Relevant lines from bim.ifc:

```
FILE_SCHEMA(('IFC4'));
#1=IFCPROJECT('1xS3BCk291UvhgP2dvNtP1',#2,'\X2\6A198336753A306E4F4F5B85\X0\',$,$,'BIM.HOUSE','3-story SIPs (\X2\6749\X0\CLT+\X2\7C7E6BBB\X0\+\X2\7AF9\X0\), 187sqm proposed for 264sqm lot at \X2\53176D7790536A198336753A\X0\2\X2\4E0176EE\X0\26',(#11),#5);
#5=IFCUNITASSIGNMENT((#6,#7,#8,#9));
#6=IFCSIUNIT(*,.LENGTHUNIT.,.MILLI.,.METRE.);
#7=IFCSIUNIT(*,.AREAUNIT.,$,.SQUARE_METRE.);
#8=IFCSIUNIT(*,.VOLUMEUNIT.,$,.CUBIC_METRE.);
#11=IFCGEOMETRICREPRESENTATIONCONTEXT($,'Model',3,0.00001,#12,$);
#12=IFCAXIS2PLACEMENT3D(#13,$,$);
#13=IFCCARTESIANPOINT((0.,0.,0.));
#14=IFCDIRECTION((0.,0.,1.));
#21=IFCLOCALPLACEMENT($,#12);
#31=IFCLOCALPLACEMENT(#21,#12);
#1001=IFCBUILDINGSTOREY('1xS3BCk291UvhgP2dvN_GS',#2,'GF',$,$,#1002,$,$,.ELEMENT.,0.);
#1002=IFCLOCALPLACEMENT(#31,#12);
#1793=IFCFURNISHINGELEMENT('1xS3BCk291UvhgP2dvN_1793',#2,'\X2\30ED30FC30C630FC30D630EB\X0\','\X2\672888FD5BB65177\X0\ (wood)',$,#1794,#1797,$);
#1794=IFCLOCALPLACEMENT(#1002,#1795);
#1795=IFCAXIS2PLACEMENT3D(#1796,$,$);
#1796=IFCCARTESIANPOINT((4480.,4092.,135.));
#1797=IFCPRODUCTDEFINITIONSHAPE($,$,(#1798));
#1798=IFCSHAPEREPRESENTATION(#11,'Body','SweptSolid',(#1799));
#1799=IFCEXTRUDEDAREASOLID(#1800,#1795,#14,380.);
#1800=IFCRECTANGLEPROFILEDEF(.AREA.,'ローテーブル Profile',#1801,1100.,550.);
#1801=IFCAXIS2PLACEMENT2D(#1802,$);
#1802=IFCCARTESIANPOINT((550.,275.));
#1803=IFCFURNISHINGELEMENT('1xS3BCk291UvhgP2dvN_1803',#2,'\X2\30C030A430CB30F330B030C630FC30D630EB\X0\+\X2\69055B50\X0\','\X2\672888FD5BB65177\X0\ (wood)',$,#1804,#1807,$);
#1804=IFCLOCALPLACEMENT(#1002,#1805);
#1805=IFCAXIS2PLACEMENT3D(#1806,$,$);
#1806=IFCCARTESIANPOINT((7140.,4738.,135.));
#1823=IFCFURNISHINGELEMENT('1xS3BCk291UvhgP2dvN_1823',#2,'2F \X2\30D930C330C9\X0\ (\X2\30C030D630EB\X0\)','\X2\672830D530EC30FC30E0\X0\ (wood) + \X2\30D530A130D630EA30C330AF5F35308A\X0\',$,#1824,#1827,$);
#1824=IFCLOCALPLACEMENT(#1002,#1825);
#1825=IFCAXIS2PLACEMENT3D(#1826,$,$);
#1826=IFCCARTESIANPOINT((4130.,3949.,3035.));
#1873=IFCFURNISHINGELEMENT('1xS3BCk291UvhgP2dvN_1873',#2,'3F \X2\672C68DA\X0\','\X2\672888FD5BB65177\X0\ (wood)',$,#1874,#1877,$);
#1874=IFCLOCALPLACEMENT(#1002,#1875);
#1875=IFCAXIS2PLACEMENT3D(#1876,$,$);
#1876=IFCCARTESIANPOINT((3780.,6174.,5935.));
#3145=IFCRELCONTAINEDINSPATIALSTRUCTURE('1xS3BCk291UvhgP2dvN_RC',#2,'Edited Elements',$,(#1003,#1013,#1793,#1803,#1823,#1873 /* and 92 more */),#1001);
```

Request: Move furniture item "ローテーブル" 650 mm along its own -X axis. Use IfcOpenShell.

```python
import ifcopenshell
import ifcopenshell.api.geometry
import ifcopenshell.util.placement
import ifcopenshell.util.unit

model = ifcopenshell.open("bim.ifc")
unit_scale = ifcopenshell.util.unit.calculate_unit_scale(model)

item = model.by_guid("1xS3BCk291UvhgP2dvN_1793")
matrix = ifcopenshell.util.placement.get_local_placement(item.ObjectPlacement)
matrix[:3, 3] -= matrix[:3, 0] * 0.65 / unit_scale
ifcopenshell.api.geometry.edit_object_placement(model, product=item, matrix=matrix, is_si=False)

print(ifcopenshell.util.placement.get_local_placement(item.ObjectPlacement).round(3) + 0.0)

model.write("bim_edited.ifc")
```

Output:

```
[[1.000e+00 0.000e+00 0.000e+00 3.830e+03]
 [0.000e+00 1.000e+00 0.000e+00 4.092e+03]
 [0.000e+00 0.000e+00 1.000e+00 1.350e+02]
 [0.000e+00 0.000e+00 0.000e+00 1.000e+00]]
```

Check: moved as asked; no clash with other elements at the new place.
